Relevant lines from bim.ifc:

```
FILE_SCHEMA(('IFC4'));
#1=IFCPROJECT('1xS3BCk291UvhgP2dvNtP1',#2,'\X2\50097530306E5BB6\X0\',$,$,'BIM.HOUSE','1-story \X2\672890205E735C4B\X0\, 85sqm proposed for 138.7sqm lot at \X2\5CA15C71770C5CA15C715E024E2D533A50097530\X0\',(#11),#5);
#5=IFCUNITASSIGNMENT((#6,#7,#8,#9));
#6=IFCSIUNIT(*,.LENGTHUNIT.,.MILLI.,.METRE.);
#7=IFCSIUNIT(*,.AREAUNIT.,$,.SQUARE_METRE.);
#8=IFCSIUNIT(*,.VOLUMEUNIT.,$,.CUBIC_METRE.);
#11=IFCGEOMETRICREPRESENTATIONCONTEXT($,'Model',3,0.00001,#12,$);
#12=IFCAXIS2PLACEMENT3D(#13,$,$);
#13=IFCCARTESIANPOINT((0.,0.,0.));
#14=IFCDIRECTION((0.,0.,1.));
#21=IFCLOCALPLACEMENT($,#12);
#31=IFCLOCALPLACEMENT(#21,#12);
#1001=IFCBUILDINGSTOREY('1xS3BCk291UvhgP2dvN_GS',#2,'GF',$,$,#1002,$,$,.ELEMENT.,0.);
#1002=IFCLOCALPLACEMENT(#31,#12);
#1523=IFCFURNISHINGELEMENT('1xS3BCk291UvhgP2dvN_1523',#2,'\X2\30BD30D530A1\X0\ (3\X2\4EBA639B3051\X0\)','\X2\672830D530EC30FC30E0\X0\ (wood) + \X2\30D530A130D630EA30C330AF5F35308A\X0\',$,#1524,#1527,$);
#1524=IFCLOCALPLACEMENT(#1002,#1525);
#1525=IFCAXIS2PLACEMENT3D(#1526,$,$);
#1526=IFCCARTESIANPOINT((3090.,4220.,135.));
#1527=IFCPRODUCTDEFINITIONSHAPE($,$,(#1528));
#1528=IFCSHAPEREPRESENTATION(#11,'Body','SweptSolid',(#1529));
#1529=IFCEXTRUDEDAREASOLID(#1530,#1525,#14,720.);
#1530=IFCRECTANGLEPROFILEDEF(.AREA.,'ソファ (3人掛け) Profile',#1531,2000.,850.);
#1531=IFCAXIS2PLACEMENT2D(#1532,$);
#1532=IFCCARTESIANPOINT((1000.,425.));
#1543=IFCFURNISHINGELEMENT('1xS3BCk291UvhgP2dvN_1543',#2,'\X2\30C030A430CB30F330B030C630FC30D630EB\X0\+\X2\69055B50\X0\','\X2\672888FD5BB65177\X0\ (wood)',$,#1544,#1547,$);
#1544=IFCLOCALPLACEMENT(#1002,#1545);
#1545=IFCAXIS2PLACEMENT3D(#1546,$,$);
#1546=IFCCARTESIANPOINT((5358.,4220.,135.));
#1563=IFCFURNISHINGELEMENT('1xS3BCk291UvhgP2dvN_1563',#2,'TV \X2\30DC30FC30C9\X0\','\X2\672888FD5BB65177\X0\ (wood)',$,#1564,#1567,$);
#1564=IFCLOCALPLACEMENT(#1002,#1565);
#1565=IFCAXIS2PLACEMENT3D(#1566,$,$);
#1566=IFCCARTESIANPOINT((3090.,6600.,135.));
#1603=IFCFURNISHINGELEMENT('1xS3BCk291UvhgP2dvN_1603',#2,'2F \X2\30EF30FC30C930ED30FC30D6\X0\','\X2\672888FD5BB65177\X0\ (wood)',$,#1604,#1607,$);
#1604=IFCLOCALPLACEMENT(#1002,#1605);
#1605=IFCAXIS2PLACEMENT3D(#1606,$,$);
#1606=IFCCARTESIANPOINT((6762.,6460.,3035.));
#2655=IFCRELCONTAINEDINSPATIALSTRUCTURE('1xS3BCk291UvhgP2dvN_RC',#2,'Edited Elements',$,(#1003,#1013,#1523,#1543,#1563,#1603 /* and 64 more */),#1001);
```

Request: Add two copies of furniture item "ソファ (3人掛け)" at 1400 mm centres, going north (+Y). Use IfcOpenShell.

```python
import numpy as np
import ifcopenshell
import ifcopenshell.api.geometry
import ifcopenshell.api.root
import ifcopenshell.util.element
import ifcopenshell.util.placement
import ifcopenshell.util.unit

model = ifcopenshell.open("bim.ifc")
unit_scale = ifcopenshell.util.unit.calculate_unit_scale(model)


def reuse_history(source, copy):
    """copy_class also copies each property set's owner history, people and application; keep the originals."""
    for rel in copy.IsDefinedBy:
        if rel.is_a("IfcRelDefinesByProperties") and (history := rel.RelatingPropertyDefinition.OwnerHistory):
            rel.RelatingPropertyDefinition.OwnerHistory = source.OwnerHistory
            ifcopenshell.util.element.remove_deep2(model, history)


source = model.by_guid("1xS3BCk291UvhgP2dvN_1523")
base = ifcopenshell.util.placement.get_local_placement(source.ObjectPlacement)
step = np.array([0.0, 1.0, 0.0]) * 1.4 / unit_scale

for i in range(1, 3):
    copy = ifcopenshell.api.root.copy_class(model, product=source)
    copy.Representation = ifcopenshell.util.element.copy_deep(
        model, source.Representation, exclude=["IfcGeometricRepresentationContext", "IfcRepresentationMap"]
    )
    reuse_history(source, copy)
    matrix = base.copy()
    matrix[:3, 3] += i * step
    print("added at", matrix[:3, 3].round(3) + 0.0)
    ifcopenshell.api.geometry.edit_object_placement(model, product=copy, matrix=matrix, is_si=False)

model.write("bim_updated.ifc")
```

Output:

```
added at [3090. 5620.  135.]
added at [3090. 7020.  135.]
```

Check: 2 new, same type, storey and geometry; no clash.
